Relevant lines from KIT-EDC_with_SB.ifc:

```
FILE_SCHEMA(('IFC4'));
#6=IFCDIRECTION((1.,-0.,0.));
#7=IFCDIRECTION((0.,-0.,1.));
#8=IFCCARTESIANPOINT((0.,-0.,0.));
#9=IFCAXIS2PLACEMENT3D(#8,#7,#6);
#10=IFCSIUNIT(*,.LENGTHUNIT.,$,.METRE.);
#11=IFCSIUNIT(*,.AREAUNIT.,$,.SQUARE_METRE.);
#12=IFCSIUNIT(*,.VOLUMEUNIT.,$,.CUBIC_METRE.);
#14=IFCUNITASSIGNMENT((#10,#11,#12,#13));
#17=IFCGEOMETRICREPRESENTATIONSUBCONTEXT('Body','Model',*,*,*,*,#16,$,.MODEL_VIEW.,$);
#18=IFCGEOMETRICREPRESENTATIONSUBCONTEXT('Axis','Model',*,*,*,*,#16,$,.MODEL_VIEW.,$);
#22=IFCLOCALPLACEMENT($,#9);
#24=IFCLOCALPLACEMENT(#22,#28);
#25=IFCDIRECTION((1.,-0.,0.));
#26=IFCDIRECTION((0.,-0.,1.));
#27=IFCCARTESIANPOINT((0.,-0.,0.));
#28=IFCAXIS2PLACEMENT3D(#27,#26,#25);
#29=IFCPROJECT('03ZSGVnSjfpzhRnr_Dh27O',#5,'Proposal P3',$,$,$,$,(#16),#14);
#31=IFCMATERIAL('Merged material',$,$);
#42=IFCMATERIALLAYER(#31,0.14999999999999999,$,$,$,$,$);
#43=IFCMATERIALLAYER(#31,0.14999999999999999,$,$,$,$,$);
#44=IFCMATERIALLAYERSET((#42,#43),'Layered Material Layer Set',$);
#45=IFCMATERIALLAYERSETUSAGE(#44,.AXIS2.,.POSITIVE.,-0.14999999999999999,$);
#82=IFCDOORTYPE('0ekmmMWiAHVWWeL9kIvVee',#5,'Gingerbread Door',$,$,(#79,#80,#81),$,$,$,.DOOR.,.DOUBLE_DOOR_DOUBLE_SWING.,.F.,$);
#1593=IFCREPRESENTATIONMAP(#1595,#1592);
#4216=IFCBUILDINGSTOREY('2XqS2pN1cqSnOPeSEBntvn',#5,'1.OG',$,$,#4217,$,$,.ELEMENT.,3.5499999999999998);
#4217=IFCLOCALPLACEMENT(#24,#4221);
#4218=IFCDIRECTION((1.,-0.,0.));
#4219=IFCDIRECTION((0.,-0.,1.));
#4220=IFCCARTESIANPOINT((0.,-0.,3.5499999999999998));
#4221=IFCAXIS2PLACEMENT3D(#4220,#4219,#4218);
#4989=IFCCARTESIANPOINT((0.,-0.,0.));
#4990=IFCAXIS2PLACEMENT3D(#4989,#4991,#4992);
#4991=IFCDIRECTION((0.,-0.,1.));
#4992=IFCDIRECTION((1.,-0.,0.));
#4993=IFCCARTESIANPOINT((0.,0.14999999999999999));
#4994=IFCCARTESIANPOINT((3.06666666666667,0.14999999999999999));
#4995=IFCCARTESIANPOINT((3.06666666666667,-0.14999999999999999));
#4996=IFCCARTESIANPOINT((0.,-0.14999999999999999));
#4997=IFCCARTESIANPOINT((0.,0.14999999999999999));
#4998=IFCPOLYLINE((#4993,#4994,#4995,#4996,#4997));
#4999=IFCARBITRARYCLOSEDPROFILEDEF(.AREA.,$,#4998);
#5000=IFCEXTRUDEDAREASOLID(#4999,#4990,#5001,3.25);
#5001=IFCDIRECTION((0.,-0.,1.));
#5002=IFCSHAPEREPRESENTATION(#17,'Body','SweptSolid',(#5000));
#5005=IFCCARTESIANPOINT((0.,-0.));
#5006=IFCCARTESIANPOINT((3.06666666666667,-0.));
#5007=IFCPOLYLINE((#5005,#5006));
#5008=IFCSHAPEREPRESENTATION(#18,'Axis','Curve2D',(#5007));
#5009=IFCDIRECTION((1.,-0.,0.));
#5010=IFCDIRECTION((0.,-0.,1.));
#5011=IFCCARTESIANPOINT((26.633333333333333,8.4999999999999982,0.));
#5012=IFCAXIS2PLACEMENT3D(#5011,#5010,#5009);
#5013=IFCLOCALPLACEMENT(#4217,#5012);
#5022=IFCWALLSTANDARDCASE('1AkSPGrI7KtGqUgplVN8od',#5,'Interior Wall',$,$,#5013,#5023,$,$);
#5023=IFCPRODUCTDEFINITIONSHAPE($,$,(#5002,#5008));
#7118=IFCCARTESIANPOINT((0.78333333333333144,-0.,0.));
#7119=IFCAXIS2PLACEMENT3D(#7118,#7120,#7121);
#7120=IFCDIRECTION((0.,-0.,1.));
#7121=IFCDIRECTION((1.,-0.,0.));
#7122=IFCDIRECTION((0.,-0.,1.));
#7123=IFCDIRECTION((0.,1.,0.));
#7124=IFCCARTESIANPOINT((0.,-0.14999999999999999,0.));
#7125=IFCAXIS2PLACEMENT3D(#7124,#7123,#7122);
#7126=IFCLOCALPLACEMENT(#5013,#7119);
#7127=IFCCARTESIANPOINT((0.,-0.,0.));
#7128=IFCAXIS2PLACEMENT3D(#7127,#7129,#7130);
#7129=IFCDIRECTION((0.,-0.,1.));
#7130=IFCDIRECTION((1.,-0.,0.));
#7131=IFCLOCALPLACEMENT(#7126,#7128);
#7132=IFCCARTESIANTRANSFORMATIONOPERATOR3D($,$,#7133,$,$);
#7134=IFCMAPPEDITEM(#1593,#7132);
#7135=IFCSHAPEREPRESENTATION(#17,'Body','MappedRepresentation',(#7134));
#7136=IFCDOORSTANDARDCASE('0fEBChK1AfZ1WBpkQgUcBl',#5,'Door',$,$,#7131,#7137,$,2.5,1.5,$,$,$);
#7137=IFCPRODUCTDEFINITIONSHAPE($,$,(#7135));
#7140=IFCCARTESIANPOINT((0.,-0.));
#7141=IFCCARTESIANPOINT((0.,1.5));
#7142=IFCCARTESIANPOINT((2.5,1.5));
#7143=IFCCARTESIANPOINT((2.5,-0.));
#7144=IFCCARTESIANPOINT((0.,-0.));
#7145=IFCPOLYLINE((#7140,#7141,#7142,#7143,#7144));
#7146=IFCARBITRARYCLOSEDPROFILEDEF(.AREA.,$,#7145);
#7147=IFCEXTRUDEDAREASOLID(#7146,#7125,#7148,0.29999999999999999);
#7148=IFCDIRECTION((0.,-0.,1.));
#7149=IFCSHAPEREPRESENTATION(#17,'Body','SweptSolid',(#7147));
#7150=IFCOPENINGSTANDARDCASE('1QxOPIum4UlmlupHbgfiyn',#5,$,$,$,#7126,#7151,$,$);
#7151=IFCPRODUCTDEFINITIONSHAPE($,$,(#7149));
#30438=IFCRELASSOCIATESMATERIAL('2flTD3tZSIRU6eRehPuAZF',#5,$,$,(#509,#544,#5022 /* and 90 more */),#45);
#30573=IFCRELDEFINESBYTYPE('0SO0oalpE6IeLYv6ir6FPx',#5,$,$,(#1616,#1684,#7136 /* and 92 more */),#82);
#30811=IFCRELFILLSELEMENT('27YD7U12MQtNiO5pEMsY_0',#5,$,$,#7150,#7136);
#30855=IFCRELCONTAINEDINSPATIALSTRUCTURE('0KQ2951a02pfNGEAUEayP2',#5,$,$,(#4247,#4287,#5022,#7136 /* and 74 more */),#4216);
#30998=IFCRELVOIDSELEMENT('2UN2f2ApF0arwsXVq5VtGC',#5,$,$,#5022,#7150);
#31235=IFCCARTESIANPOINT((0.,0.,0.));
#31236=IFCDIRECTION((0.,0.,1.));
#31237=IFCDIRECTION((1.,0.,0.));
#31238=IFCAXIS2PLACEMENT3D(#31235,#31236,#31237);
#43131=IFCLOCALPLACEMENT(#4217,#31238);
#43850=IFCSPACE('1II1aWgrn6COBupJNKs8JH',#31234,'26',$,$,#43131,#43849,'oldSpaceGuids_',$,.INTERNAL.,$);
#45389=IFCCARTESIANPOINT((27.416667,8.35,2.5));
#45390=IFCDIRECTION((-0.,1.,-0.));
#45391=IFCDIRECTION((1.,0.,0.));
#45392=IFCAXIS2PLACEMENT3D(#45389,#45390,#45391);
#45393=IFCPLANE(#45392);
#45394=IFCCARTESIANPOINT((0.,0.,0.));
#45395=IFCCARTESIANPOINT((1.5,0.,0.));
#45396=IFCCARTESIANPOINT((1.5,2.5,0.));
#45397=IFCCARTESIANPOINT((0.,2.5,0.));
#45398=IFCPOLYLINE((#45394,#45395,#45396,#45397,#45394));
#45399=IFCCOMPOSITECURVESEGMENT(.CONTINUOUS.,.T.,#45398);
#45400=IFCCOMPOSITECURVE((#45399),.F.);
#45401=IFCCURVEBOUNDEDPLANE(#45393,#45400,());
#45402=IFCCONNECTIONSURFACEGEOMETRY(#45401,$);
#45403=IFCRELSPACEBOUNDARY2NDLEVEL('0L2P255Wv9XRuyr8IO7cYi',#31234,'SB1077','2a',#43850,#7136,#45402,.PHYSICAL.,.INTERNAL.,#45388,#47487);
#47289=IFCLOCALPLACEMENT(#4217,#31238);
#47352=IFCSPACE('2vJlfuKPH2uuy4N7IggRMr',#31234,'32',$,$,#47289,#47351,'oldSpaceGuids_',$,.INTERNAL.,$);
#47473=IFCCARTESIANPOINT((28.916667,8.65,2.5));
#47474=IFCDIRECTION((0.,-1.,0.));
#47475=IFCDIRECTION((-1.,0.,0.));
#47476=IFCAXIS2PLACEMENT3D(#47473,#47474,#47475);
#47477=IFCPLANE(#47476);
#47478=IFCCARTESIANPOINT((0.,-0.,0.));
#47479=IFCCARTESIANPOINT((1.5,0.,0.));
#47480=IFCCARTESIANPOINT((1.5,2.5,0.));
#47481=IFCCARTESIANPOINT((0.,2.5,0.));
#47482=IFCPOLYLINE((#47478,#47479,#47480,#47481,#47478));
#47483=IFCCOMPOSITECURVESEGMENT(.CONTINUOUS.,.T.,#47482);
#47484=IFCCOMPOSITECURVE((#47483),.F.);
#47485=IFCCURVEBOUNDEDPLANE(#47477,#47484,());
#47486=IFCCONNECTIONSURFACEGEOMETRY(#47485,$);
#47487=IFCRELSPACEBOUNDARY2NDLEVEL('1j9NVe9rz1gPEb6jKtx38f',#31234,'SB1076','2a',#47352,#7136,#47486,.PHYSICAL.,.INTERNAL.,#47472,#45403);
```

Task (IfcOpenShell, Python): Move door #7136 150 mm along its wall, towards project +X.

```python
import numpy as np
import ifcopenshell
import ifcopenshell.api.geometry
import ifcopenshell.util.placement
import ifcopenshell.util.unit

model = ifcopenshell.open("KIT-EDC_with_SB.ifc")
unit_scale = ifcopenshell.util.unit.calculate_unit_scale(model)

door = model.by_guid("0fEBChK1AfZ1WBpkQgUcBl")
opening = door.FillsVoids[0].RelatingOpeningElement
wall = opening.VoidsElements[0].RelatingBuildingElement

wall_matrix = ifcopenshell.util.placement.get_local_placement(wall.ObjectPlacement)
shift = wall_matrix[:3, 0] * 0.15 / unit_scale
before = ifcopenshell.util.placement.get_local_placement(door.ObjectPlacement)[:3, 3].copy()

# The door is placed relative to its opening, so it follows when the opening moves.
matrix = ifcopenshell.util.placement.get_local_placement(opening.ObjectPlacement)
matrix[:3, 3] += shift
ifcopenshell.api.geometry.edit_object_placement(
    model, product=opening, matrix=matrix, is_si=False, should_transform_children=True
)

# Space boundary surfaces are stored in each space's coordinates; move them too.
for rel in door.ProvidesBoundaries:
    if not rel.ConnectionGeometry:
        continue
    surface = rel.ConnectionGeometry.SurfaceOnRelatingElement.BasisSurface
    space_matrix = ifcopenshell.util.placement.get_local_placement(rel.RelatingSpace.ObjectPlacement)
    point = np.array(surface.Position.Location.Coordinates) + space_matrix[:3, :3].T @ shift
    surface.Position = model.createIfcAxis2Placement3D(
        model.createIfcCartesianPoint(point.tolist()), surface.Position.Axis, surface.Position.RefDirection
    )

after = ifcopenshell.util.placement.get_local_placement(door.ObjectPlacement)[:3, 3]
print("door moved by", (after - before).round(3) + 0.0)

model.write("KIT-EDC_with_SB-out.ifc")
```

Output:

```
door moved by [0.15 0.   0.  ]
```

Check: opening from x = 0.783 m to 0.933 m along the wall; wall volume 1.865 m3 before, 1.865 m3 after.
